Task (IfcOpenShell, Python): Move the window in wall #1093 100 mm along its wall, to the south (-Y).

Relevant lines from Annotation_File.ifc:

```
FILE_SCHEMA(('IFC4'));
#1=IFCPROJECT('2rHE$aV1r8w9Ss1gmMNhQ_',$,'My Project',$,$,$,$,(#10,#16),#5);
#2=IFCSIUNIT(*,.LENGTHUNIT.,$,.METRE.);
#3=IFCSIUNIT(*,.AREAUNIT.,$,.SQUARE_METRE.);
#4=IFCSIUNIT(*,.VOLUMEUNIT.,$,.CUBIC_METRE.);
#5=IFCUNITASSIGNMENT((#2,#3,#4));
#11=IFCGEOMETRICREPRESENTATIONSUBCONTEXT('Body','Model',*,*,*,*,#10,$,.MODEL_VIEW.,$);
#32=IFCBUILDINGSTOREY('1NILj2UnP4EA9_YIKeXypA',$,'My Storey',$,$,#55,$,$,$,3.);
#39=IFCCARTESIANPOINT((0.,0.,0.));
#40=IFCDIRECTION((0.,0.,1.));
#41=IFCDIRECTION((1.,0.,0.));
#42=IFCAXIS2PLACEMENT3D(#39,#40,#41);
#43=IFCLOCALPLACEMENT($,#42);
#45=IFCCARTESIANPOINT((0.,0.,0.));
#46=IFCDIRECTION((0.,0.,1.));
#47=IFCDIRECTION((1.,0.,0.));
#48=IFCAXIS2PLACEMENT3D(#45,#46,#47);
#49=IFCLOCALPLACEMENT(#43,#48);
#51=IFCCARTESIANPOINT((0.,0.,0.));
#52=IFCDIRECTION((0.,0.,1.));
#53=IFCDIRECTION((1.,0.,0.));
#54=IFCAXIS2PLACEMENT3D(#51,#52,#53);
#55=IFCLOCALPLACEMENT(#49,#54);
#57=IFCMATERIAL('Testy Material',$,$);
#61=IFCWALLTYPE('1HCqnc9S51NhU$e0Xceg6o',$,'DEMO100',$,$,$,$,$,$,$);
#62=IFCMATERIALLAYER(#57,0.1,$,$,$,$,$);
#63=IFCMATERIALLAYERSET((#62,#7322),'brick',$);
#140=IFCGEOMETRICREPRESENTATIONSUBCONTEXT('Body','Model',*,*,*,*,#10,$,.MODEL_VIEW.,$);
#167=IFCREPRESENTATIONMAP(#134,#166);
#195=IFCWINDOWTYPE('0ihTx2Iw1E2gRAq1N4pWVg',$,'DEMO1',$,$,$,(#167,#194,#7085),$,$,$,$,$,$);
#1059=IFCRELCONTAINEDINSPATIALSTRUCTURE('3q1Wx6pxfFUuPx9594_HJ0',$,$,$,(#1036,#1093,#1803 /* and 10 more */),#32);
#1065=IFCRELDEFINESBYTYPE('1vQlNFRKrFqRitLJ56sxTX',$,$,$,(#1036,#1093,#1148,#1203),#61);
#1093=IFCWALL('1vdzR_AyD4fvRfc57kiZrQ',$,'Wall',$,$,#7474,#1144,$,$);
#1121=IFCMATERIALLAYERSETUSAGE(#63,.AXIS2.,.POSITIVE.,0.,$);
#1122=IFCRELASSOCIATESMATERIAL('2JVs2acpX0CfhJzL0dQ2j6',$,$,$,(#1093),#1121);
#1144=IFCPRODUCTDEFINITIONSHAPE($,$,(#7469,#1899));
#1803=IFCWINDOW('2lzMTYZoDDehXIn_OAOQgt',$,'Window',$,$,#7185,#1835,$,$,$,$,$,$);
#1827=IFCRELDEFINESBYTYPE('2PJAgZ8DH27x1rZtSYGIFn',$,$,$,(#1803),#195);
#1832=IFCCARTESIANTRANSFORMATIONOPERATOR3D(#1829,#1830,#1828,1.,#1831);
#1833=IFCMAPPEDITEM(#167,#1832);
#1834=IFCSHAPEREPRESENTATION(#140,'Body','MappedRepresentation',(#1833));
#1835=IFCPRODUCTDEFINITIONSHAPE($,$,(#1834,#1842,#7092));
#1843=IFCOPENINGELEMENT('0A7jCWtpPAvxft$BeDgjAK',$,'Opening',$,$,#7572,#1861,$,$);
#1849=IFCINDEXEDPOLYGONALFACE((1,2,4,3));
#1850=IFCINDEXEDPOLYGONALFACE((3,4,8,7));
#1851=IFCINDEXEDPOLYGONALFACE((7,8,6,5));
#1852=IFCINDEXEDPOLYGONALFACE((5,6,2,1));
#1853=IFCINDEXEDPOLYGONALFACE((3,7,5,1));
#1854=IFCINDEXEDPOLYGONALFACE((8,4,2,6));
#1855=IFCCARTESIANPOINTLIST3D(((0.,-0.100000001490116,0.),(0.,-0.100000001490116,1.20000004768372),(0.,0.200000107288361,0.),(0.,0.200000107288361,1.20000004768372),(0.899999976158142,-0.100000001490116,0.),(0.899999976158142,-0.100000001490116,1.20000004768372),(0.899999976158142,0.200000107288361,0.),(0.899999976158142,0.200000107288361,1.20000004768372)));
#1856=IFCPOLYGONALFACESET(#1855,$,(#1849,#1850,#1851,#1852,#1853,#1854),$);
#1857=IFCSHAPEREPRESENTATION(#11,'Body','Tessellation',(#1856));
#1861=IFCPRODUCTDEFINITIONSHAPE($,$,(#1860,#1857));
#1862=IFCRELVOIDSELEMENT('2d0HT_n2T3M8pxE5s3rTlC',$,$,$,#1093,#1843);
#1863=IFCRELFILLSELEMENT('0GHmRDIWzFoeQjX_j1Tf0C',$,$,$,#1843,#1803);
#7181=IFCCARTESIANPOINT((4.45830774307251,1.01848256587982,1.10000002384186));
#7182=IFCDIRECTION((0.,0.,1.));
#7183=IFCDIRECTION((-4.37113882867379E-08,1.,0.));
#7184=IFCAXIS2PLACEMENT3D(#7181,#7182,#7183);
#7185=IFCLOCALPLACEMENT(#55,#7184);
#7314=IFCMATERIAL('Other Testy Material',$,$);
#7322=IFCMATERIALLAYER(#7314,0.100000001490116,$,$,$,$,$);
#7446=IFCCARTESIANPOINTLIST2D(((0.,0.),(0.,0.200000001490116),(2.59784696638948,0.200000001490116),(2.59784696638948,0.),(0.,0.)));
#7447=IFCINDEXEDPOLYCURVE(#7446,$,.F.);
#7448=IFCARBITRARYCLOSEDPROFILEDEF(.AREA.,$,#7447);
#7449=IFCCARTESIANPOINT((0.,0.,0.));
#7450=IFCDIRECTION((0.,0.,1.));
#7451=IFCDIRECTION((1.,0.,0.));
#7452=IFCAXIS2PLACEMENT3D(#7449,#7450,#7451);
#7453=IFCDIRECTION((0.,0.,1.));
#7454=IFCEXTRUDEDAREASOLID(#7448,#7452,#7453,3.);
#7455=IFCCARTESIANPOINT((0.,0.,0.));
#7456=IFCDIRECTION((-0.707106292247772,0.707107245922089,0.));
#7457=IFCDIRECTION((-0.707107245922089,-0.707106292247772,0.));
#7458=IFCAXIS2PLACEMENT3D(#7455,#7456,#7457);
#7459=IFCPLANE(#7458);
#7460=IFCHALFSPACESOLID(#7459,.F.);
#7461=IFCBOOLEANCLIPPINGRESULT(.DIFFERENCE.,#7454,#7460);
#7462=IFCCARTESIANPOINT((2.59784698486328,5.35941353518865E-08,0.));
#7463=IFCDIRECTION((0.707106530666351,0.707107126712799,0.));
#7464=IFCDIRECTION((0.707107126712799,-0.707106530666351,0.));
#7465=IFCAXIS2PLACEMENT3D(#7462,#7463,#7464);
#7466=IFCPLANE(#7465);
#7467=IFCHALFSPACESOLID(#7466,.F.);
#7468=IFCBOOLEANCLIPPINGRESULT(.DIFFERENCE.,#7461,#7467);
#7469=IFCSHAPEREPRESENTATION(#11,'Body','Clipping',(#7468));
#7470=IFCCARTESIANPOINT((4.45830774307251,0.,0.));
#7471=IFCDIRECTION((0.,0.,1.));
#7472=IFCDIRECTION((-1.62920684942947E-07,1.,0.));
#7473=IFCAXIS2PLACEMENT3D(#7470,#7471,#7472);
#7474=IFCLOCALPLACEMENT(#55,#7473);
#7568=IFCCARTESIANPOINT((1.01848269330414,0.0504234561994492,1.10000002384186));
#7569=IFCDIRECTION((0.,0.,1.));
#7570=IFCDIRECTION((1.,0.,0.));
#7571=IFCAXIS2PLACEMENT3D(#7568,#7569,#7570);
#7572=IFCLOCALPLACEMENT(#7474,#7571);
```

```python
import ifcopenshell
import ifcopenshell.api.geometry
import ifcopenshell.util.placement
import ifcopenshell.util.unit

model = ifcopenshell.open("Annotation_File.ifc")
unit_scale = ifcopenshell.util.unit.calculate_unit_scale(model)

window = model.by_id(1803)
opening = window.FillsVoids[0].RelatingOpeningElement
wall = opening.VoidsElements[0].RelatingBuildingElement

wall_matrix = ifcopenshell.util.placement.get_local_placement(wall.ObjectPlacement)
shift = wall_matrix[:3, 0] * -0.1 / unit_scale
before = ifcopenshell.util.placement.get_local_placement(window.ObjectPlacement)[:3, 3].copy()

# The window is not placed relative to its opening, so move both.
for product in (opening, window):
    matrix = ifcopenshell.util.placement.get_local_placement(product.ObjectPlacement)
    matrix[:3, 3] += shift
    ifcopenshell.api.geometry.edit_object_placement(model, product=product, matrix=matrix, is_si=False)

after = ifcopenshell.util.placement.get_local_placement(window.ObjectPlacement)[:3, 3]
print("window moved by", (after - before).round(3) + 0.0)

model.write("Annotation_File_rev.ifc")
```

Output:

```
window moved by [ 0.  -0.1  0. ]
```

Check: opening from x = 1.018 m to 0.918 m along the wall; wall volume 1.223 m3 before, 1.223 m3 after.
